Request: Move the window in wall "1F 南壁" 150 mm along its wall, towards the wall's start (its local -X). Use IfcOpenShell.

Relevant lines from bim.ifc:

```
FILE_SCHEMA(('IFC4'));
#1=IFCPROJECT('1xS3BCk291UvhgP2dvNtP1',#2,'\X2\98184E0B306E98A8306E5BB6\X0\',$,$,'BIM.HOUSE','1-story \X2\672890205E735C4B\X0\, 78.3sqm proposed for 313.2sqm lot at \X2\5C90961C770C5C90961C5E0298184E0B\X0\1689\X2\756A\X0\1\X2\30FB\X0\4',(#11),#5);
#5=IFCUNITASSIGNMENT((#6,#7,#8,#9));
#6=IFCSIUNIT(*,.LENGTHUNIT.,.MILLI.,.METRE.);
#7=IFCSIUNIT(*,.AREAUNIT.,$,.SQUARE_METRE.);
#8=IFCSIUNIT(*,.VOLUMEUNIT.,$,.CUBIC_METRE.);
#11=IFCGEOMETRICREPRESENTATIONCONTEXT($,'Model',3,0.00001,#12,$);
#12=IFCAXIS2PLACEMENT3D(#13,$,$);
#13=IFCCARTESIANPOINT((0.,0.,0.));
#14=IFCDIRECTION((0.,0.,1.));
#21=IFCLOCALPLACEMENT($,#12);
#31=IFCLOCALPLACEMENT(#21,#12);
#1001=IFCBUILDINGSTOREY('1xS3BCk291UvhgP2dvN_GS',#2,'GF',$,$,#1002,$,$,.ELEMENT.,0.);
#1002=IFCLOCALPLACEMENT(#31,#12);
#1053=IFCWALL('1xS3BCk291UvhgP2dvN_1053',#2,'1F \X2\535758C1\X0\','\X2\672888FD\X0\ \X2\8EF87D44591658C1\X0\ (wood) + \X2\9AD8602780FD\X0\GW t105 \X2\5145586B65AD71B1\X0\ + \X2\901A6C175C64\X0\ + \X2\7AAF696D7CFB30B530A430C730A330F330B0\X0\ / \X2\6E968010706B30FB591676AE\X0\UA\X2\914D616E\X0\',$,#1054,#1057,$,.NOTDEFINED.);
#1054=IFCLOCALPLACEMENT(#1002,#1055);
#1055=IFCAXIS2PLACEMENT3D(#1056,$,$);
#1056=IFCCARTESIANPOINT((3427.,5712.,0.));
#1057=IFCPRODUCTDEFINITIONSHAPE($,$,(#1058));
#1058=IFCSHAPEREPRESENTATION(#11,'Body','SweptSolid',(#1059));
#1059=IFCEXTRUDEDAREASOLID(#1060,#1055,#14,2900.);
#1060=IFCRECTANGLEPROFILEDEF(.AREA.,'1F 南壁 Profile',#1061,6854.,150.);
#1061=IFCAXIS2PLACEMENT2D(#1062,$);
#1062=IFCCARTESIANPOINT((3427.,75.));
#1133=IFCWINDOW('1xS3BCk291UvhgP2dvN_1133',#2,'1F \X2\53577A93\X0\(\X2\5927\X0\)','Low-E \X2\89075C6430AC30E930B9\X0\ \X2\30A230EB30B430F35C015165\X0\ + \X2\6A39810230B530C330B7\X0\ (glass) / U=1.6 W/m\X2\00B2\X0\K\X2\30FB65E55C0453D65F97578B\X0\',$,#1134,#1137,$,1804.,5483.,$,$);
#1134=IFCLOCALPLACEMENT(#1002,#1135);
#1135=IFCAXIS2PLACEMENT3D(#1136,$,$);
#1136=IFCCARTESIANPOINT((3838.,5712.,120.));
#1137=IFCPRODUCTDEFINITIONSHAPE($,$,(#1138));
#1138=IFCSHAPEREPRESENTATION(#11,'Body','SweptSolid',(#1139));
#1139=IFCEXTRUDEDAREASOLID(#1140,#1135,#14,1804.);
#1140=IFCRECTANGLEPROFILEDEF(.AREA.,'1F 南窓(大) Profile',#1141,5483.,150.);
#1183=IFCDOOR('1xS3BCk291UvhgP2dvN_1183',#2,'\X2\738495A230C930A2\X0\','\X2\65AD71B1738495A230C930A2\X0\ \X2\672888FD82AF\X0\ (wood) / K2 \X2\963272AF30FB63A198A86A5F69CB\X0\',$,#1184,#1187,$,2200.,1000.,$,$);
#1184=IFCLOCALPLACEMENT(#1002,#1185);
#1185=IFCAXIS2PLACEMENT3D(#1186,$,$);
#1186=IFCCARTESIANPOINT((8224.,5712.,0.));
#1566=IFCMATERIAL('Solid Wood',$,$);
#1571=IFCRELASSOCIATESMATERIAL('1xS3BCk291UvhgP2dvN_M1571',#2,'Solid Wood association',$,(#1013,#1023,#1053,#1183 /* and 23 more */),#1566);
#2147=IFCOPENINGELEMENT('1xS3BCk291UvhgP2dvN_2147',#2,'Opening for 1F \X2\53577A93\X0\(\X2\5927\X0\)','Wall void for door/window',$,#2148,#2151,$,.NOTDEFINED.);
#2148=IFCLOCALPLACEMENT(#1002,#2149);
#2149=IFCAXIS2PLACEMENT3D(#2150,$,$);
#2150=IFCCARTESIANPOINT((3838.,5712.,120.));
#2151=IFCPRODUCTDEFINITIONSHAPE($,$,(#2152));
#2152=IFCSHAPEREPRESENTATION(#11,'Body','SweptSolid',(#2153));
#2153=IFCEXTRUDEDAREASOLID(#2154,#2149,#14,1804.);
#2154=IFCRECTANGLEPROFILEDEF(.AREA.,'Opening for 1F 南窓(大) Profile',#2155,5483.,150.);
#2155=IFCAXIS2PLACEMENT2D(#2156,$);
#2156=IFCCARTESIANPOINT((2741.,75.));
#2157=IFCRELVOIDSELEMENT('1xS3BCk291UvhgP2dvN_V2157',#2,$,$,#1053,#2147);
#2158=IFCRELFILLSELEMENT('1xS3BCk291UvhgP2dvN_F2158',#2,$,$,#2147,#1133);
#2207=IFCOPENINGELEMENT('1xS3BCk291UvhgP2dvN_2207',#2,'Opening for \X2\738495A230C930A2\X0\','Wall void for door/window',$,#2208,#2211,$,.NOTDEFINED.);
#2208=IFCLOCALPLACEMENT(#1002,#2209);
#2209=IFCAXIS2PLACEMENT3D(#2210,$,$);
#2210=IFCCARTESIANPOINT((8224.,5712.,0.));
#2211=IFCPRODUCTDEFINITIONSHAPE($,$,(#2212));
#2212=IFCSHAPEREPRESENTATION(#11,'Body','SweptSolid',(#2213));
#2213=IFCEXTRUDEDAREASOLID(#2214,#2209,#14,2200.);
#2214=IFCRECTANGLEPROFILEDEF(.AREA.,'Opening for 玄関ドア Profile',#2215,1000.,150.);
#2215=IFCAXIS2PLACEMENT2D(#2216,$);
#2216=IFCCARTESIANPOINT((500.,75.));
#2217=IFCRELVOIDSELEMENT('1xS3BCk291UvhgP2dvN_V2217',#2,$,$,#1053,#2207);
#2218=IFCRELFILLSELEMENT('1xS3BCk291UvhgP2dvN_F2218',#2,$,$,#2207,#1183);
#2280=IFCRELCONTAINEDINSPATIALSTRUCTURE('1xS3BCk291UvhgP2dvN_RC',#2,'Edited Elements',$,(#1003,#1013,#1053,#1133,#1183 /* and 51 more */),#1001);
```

```python
import ifcopenshell
import ifcopenshell.api.geometry
import ifcopenshell.util.placement
import ifcopenshell.util.unit

model = ifcopenshell.open("bim.ifc")
unit_scale = ifcopenshell.util.unit.calculate_unit_scale(model)

window = model.by_id(1133)
opening = window.FillsVoids[0].RelatingOpeningElement
wall = opening.VoidsElements[0].RelatingBuildingElement

wall_matrix = ifcopenshell.util.placement.get_local_placement(wall.ObjectPlacement)
shift = wall_matrix[:3, 0] * -0.15 / unit_scale
before = ifcopenshell.util.placement.get_local_placement(window.ObjectPlacement)[:3, 3].copy()

# The window is not placed relative to its opening, so move both.
for product in (opening, window):
    matrix = ifcopenshell.util.placement.get_local_placement(product.ObjectPlacement)
    matrix[:3, 3] += shift
    ifcopenshell.api.geometry.edit_object_placement(model, product=product, matrix=matrix, is_si=False)

after = ifcopenshell.util.placement.get_local_placement(window.ObjectPlacement)[:3, 3]
print("window moved by", (after - before).round(3) + 0.0)

model.write("bim-out.ifc")
```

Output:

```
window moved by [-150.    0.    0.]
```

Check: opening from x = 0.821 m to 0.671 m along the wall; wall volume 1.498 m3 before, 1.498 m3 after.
